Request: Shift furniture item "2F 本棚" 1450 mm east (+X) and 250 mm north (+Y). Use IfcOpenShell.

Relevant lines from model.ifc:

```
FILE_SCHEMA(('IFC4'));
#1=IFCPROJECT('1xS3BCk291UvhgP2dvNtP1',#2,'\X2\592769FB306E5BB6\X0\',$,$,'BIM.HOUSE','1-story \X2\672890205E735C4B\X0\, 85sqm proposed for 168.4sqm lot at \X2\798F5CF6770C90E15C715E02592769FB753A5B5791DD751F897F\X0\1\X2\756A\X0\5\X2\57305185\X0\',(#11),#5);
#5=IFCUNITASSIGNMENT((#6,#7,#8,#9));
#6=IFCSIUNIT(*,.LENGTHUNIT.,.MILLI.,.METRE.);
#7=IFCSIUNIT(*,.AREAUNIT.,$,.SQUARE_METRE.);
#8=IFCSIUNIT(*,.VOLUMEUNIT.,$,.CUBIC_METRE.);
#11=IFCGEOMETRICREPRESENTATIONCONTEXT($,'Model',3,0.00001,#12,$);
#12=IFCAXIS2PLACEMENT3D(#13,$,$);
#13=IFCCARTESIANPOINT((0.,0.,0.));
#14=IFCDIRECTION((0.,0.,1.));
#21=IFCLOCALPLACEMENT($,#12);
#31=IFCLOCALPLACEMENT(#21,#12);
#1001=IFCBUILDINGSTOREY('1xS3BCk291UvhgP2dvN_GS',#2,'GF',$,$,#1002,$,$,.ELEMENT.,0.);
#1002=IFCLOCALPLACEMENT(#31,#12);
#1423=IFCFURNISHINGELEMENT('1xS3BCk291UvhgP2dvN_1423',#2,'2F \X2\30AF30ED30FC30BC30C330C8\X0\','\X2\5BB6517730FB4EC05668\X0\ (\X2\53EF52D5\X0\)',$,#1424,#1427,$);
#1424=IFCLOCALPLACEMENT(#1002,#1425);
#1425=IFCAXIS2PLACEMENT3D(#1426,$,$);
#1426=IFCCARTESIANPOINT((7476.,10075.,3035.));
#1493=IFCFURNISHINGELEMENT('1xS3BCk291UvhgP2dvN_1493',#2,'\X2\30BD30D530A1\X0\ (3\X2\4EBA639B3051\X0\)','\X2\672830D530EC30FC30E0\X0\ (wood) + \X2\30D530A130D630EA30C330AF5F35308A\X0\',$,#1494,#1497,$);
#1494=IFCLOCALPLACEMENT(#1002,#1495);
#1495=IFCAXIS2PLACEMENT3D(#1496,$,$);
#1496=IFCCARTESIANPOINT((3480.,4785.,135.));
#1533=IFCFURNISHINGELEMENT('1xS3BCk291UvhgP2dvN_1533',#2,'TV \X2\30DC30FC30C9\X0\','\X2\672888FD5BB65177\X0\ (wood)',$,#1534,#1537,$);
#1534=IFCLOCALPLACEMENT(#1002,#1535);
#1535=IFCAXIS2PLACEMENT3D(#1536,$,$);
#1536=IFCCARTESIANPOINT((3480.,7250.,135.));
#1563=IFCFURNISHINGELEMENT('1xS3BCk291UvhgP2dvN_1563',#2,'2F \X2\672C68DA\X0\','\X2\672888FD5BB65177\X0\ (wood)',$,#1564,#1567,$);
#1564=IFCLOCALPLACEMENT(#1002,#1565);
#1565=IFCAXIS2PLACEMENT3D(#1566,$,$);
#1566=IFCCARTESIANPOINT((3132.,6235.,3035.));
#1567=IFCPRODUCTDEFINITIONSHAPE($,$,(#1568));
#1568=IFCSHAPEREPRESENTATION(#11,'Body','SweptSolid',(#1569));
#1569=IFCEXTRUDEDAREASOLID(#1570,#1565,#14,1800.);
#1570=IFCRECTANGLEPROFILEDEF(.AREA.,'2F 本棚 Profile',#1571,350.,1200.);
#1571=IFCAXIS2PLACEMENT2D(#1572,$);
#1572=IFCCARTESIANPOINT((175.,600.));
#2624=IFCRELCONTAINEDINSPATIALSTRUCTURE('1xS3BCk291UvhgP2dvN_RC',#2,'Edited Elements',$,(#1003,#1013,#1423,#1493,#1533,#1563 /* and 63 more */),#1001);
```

```python
import ifcopenshell
import ifcopenshell.api.geometry
import ifcopenshell.util.placement

model = ifcopenshell.open("model.ifc")

item = model.by_id(1563)
matrix = ifcopenshell.util.placement.get_local_placement(item.ObjectPlacement)
matrix[0, 3] += 1450.0
matrix[1, 3] += 250.0
ifcopenshell.api.geometry.edit_object_placement(model, product=item, matrix=matrix, is_si=False)

print(ifcopenshell.util.placement.get_local_placement(item.ObjectPlacement).round(3) + 0.0)

model.write("model_edited.ifc")
```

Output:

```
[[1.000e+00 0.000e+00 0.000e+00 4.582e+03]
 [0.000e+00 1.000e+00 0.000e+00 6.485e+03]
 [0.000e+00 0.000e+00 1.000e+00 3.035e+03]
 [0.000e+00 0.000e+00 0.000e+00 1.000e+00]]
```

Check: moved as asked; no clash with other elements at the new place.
